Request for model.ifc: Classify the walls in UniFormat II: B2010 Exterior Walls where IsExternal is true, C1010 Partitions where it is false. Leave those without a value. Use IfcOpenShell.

First a look at what the model holds.

```python
import ifcopenshell
import ifcopenshell.util.element

model = ifcopenshell.open("model.ifc")
print(model.schema)
print("classifications:", [c.Name for c in model.by_type("IfcClassification")])
values = [ifcopenshell.util.element.get_pset(e, "Pset_WallCommon", "IsExternal") for e in model.by_type("IfcWall")]
for value in (True, False, None):
    print("IsExternal", value, values.count(value))
```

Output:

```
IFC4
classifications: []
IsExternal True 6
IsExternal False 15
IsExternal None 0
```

```python
import ifcopenshell
import ifcopenshell.api.classification
import ifcopenshell.util.element

model = ifcopenshell.open("model.ifc")

system = ifcopenshell.api.classification.add_classification(model, classification="UniFormat II")

walls = model.by_type("IfcWall")
external = {e: ifcopenshell.util.element.get_pset(e, "Pset_WallCommon", "IsExternal") for e in walls}
for flag, code, name in ((True, "B2010", "Exterior Walls"), (False, "C1010", "Partitions")):
    products = [e for e in walls if external[e] is flag]
    ifcopenshell.api.classification.add_reference(
        model, products=products, classification=system, identification=code, name=name
    )
    print(code, len(products))

model.write("model_edited.ifc")
```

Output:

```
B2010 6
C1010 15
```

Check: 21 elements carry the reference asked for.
